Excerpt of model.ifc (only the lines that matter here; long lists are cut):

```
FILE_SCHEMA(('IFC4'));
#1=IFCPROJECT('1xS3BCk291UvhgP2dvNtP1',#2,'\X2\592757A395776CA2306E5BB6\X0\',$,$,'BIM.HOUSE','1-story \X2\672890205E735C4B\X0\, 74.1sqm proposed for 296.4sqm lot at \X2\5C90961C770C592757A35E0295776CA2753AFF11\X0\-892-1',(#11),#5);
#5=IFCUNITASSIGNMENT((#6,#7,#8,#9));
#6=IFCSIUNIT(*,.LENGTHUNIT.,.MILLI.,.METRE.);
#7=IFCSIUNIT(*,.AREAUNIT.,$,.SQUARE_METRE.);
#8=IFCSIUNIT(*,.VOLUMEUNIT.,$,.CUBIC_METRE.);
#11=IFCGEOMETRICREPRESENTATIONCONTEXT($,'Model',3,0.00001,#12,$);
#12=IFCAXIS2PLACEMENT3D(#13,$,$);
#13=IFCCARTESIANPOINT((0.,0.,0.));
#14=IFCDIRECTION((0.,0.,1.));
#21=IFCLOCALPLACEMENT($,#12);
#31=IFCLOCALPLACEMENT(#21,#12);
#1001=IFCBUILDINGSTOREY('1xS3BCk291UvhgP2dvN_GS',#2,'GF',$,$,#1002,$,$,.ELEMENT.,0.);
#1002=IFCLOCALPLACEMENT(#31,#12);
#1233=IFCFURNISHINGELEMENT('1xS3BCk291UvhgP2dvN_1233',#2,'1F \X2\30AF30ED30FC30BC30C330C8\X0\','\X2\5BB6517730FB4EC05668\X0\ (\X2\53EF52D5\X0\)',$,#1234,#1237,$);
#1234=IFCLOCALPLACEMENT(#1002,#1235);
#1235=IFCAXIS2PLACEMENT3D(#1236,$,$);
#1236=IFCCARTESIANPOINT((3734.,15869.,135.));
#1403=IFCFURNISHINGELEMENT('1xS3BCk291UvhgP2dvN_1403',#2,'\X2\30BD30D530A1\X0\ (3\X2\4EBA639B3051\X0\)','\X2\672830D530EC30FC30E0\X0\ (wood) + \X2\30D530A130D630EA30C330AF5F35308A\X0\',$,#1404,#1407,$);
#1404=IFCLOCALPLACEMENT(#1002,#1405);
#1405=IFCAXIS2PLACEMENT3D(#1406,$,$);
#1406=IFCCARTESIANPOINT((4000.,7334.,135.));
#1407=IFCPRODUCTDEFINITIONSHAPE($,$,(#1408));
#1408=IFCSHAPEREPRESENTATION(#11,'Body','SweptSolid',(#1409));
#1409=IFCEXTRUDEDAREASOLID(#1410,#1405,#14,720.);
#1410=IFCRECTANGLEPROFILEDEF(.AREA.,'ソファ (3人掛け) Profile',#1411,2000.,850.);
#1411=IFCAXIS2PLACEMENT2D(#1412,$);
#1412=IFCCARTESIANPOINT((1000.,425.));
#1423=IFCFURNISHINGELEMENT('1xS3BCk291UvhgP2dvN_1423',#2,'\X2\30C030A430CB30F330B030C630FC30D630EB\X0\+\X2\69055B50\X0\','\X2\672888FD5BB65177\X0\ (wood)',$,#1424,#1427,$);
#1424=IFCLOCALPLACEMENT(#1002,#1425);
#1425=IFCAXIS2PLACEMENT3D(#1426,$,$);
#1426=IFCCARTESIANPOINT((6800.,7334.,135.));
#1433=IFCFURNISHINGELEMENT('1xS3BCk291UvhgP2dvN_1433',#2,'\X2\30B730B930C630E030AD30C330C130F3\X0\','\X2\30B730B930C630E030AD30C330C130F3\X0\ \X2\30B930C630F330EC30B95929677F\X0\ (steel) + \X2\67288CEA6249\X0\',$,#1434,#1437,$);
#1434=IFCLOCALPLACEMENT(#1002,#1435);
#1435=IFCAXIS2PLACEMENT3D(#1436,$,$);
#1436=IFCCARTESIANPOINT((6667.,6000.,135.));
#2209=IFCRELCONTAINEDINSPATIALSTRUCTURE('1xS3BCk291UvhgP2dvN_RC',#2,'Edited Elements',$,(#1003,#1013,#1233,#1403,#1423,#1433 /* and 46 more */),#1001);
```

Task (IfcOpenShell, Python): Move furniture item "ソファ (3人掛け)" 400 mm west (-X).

```python
import ifcopenshell
import ifcopenshell.api.geometry
import ifcopenshell.util.placement
import ifcopenshell.util.unit

model = ifcopenshell.open("model.ifc")
unit_scale = ifcopenshell.util.unit.calculate_unit_scale(model)

item = model.by_guid("1xS3BCk291UvhgP2dvN_1403")
matrix = ifcopenshell.util.placement.get_local_placement(item.ObjectPlacement)
matrix[0, 3] -= 0.4 / unit_scale
ifcopenshell.api.geometry.edit_object_placement(model, product=item, matrix=matrix, is_si=False)

print(ifcopenshell.util.placement.get_local_placement(item.ObjectPlacement).round(3) + 0.0)

model.write("model_updated.ifc")
```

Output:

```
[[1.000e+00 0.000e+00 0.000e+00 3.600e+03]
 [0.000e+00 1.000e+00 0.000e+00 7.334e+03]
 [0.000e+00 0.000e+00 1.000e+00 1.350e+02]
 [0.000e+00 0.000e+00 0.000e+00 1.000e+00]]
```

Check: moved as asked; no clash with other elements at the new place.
